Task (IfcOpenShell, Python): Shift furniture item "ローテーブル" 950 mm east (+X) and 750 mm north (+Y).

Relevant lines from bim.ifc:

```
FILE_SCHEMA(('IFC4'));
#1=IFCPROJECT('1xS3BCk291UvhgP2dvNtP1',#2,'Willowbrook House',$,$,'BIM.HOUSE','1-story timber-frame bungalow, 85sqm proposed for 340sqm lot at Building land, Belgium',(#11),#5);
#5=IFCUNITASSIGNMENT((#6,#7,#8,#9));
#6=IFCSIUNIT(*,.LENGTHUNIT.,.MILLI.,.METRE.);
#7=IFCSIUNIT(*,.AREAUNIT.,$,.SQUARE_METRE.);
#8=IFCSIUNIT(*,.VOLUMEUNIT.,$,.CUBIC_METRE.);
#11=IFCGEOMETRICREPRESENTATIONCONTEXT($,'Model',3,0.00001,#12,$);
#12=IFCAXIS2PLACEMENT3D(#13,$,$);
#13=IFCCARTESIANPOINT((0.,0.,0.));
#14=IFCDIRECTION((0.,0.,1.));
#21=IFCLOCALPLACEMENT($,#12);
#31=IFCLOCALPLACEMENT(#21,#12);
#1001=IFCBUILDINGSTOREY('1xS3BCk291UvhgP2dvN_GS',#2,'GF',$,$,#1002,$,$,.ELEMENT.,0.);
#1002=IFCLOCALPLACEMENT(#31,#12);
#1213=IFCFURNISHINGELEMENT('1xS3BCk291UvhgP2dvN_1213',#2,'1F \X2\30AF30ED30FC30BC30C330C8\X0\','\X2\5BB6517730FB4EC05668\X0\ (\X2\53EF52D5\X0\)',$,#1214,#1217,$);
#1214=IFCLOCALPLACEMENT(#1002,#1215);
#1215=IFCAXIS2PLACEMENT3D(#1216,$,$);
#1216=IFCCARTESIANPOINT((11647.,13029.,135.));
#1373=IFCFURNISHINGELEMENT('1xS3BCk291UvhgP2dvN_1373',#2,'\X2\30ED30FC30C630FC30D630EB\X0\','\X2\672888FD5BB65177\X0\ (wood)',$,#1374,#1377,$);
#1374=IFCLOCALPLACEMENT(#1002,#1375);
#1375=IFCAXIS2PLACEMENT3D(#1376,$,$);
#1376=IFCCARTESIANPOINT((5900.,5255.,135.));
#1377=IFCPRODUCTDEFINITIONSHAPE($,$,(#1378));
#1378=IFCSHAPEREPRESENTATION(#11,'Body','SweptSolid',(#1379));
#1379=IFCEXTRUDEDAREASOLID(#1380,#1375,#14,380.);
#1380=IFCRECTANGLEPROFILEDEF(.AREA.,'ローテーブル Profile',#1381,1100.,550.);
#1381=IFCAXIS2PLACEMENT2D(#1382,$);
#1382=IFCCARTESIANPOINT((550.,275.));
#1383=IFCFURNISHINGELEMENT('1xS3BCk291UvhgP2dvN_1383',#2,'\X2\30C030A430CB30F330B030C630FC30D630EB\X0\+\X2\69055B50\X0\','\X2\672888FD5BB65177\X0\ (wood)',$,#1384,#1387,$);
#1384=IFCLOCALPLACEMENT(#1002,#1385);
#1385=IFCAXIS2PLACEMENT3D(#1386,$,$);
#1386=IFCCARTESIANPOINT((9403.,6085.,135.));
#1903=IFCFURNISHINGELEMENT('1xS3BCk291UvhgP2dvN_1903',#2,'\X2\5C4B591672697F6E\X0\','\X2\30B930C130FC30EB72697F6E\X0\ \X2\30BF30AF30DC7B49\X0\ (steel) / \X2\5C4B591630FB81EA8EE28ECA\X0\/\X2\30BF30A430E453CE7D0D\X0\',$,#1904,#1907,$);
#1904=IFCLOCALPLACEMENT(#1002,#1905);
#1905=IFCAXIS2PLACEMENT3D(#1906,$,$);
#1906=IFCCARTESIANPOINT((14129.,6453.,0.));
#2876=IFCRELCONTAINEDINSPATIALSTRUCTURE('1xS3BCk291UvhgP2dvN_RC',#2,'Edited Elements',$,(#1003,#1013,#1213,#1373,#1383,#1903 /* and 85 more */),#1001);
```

```python
import ifcopenshell
import ifcopenshell.api.geometry
import ifcopenshell.util.placement
import ifcopenshell.util.unit

model = ifcopenshell.open("bim.ifc")
unit_scale = ifcopenshell.util.unit.calculate_unit_scale(model)

item = model.by_guid("1xS3BCk291UvhgP2dvN_1373")
matrix = ifcopenshell.util.placement.get_local_placement(item.ObjectPlacement)
matrix[0, 3] += 0.95 / unit_scale
matrix[1, 3] += 0.75 / unit_scale
ifcopenshell.api.geometry.edit_object_placement(model, product=item, matrix=matrix, is_si=False)

print(ifcopenshell.util.placement.get_local_placement(item.ObjectPlacement).round(3) + 0.0)

model.write("bim_edited.ifc")
```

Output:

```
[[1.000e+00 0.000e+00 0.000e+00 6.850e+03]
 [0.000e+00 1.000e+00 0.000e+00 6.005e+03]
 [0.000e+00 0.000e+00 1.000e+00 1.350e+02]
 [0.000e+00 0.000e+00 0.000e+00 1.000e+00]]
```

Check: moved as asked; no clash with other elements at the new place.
